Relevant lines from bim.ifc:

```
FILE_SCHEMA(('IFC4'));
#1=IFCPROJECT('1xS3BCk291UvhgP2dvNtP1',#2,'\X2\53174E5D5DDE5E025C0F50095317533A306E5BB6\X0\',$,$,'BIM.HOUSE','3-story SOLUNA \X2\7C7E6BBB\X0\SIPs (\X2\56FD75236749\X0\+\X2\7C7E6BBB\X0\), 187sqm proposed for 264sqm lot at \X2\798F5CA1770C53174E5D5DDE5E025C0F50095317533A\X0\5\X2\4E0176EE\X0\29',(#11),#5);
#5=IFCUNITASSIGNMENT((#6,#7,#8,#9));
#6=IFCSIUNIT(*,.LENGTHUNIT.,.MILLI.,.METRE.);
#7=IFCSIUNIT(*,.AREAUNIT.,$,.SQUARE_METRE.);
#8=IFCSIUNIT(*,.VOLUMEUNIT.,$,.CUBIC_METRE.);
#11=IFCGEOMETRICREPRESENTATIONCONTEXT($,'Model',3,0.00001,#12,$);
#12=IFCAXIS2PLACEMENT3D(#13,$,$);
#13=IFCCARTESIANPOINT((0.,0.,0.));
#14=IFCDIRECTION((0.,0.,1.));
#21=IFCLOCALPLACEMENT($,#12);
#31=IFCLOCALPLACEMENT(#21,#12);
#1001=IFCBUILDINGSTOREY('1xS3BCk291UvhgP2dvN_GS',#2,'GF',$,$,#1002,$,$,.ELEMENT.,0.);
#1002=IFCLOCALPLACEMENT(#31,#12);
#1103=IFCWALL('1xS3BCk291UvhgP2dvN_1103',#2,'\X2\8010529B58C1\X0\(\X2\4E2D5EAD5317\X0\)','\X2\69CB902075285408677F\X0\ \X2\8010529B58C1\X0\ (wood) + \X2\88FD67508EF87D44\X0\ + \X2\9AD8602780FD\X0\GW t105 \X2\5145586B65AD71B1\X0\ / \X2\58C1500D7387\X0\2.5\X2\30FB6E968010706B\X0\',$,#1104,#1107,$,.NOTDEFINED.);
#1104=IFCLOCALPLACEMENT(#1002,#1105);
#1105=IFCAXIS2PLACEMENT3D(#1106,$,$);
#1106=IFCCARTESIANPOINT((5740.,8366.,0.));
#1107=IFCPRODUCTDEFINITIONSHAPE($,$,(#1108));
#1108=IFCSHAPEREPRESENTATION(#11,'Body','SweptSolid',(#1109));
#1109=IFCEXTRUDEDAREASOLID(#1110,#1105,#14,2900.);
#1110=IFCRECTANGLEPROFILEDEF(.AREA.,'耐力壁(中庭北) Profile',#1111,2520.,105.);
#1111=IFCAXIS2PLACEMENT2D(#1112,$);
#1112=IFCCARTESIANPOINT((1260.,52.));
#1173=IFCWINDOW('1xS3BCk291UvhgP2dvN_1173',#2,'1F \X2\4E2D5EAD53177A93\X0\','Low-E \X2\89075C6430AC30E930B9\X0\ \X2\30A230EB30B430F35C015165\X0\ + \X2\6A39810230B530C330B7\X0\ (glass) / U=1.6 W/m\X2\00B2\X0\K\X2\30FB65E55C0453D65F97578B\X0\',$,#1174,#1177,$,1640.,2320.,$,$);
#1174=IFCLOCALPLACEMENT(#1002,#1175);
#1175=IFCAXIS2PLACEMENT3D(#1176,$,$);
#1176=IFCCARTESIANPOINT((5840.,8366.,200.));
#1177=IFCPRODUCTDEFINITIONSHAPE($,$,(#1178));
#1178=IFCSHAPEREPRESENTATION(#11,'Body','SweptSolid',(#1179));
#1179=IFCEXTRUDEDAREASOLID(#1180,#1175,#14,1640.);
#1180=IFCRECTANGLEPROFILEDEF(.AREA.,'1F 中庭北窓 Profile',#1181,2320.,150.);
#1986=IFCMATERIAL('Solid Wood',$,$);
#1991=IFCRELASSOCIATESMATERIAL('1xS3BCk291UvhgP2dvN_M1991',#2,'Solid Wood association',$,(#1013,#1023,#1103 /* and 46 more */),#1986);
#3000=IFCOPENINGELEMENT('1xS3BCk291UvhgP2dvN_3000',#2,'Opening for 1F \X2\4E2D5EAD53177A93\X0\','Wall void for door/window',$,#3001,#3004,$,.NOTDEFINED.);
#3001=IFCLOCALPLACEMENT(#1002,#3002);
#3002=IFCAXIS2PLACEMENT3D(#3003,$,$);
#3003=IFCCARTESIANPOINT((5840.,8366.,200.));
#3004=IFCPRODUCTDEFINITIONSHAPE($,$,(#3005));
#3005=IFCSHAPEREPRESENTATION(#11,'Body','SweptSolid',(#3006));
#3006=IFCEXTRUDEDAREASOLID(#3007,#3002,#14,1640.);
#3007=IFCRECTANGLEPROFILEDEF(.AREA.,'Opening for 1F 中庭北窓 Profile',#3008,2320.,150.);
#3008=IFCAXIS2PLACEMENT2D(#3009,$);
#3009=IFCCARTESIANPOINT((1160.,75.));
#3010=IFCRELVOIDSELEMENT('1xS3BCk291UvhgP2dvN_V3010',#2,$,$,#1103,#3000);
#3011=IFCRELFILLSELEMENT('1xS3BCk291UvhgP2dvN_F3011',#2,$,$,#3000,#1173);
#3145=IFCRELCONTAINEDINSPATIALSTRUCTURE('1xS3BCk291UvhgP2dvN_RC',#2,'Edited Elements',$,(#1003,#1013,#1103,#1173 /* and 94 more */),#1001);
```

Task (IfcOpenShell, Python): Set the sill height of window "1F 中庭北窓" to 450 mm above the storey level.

```python
import numpy as np
import ifcopenshell
import ifcopenshell.api.geometry
import ifcopenshell.geom
import ifcopenshell.util.element
import ifcopenshell.util.placement
import ifcopenshell.util.shape
import ifcopenshell.util.unit

model = ifcopenshell.open("bim.ifc")
unit_scale = ifcopenshell.util.unit.calculate_unit_scale(model)

window = model.by_id(1173)
opening = window.FillsVoids[0].RelatingOpeningElement
storey = ifcopenshell.util.element.get_container(window, ifc_class="IfcBuildingStorey")
level = ifcopenshell.util.placement.get_local_placement(storey.ObjectPlacement)[2, 3]

# The opening's origin need not be at the sill, so measure its lowest point.
shape = ifcopenshell.geom.create_shape(ifcopenshell.geom.settings(), opening)
bottom = ifcopenshell.util.shape.get_shape_bottom_elevation(shape, shape.geometry) / unit_scale
dz = level + 0.45 / unit_scale - bottom

shift = np.array([0.0, 0.0, dz])
# The window is not placed relative to its opening, so move both.
for product in (opening, window):
    matrix = ifcopenshell.util.placement.get_local_placement(product.ObjectPlacement)
    matrix[:3, 3] += shift
    ifcopenshell.api.geometry.edit_object_placement(model, product=product, matrix=matrix, is_si=False)

print(f"moved by {dz * unit_scale:+.3f} m")

model.write("bim_rev.ifc")
```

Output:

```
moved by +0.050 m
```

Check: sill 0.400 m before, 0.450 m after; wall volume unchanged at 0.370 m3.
